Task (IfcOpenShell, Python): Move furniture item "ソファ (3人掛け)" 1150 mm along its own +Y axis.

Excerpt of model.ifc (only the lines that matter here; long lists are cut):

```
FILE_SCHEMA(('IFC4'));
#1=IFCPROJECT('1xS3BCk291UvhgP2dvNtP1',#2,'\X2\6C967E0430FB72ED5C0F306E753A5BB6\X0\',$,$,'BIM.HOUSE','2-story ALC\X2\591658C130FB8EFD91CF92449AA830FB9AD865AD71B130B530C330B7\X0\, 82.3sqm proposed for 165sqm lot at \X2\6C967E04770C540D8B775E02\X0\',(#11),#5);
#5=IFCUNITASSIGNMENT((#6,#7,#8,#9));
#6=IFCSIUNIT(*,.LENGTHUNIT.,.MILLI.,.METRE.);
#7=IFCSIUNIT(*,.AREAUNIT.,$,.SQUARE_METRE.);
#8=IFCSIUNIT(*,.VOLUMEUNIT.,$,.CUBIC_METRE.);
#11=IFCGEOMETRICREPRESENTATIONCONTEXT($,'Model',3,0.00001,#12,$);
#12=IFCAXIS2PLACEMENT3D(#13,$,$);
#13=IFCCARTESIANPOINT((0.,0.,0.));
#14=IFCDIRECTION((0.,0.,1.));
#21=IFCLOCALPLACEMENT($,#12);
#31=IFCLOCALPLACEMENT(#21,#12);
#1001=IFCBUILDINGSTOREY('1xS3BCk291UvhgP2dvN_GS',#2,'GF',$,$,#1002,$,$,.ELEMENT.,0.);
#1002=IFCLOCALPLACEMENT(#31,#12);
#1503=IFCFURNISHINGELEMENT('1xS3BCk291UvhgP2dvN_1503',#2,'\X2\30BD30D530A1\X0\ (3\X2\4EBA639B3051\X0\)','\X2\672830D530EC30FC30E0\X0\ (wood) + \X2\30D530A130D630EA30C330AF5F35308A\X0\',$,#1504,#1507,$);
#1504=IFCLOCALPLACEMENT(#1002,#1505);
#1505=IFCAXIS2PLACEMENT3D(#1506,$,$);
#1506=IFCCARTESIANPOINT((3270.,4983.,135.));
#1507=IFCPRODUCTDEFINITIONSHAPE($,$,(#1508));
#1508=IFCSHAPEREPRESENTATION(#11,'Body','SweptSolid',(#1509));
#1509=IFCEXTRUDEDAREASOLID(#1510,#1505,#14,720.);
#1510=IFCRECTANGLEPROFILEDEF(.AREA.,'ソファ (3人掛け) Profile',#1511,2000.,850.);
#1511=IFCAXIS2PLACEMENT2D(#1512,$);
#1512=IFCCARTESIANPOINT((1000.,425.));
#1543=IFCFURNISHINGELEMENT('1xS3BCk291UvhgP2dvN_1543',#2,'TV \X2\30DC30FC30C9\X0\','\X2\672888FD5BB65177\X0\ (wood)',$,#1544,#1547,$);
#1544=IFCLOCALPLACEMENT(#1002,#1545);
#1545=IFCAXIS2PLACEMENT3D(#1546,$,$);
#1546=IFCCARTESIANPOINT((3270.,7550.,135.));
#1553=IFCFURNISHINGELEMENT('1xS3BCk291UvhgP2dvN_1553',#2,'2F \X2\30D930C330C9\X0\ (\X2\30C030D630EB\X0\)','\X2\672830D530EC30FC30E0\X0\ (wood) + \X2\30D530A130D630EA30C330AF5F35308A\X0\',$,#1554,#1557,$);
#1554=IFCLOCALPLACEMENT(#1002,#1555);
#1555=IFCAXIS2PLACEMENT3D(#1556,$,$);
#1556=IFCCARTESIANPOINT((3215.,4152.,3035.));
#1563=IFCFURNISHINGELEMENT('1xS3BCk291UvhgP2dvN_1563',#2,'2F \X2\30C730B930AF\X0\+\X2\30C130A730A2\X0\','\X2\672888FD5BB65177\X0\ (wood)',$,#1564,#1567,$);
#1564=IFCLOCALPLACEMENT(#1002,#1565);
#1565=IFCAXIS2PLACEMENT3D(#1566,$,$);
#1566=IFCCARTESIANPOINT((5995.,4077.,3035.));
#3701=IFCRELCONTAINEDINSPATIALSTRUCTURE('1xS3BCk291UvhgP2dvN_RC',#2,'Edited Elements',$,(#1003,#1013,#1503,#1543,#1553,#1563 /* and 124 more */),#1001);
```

```python
import ifcopenshell
import ifcopenshell.api.geometry
import ifcopenshell.util.placement

model = ifcopenshell.open("model.ifc")

item = model.by_guid("1xS3BCk291UvhgP2dvN_1503")
matrix = ifcopenshell.util.placement.get_local_placement(item.ObjectPlacement)
matrix[:3, 3] += matrix[:3, 1] * 1150.0
ifcopenshell.api.geometry.edit_object_placement(model, product=item, matrix=matrix, is_si=False)

print(ifcopenshell.util.placement.get_local_placement(item.ObjectPlacement).round(3) + 0.0)

model.write("model_updated.ifc")
```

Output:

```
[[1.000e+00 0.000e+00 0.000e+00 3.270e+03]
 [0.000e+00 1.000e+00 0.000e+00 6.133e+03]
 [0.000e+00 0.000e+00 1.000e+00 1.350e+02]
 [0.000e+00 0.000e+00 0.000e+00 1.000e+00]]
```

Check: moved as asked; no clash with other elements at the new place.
